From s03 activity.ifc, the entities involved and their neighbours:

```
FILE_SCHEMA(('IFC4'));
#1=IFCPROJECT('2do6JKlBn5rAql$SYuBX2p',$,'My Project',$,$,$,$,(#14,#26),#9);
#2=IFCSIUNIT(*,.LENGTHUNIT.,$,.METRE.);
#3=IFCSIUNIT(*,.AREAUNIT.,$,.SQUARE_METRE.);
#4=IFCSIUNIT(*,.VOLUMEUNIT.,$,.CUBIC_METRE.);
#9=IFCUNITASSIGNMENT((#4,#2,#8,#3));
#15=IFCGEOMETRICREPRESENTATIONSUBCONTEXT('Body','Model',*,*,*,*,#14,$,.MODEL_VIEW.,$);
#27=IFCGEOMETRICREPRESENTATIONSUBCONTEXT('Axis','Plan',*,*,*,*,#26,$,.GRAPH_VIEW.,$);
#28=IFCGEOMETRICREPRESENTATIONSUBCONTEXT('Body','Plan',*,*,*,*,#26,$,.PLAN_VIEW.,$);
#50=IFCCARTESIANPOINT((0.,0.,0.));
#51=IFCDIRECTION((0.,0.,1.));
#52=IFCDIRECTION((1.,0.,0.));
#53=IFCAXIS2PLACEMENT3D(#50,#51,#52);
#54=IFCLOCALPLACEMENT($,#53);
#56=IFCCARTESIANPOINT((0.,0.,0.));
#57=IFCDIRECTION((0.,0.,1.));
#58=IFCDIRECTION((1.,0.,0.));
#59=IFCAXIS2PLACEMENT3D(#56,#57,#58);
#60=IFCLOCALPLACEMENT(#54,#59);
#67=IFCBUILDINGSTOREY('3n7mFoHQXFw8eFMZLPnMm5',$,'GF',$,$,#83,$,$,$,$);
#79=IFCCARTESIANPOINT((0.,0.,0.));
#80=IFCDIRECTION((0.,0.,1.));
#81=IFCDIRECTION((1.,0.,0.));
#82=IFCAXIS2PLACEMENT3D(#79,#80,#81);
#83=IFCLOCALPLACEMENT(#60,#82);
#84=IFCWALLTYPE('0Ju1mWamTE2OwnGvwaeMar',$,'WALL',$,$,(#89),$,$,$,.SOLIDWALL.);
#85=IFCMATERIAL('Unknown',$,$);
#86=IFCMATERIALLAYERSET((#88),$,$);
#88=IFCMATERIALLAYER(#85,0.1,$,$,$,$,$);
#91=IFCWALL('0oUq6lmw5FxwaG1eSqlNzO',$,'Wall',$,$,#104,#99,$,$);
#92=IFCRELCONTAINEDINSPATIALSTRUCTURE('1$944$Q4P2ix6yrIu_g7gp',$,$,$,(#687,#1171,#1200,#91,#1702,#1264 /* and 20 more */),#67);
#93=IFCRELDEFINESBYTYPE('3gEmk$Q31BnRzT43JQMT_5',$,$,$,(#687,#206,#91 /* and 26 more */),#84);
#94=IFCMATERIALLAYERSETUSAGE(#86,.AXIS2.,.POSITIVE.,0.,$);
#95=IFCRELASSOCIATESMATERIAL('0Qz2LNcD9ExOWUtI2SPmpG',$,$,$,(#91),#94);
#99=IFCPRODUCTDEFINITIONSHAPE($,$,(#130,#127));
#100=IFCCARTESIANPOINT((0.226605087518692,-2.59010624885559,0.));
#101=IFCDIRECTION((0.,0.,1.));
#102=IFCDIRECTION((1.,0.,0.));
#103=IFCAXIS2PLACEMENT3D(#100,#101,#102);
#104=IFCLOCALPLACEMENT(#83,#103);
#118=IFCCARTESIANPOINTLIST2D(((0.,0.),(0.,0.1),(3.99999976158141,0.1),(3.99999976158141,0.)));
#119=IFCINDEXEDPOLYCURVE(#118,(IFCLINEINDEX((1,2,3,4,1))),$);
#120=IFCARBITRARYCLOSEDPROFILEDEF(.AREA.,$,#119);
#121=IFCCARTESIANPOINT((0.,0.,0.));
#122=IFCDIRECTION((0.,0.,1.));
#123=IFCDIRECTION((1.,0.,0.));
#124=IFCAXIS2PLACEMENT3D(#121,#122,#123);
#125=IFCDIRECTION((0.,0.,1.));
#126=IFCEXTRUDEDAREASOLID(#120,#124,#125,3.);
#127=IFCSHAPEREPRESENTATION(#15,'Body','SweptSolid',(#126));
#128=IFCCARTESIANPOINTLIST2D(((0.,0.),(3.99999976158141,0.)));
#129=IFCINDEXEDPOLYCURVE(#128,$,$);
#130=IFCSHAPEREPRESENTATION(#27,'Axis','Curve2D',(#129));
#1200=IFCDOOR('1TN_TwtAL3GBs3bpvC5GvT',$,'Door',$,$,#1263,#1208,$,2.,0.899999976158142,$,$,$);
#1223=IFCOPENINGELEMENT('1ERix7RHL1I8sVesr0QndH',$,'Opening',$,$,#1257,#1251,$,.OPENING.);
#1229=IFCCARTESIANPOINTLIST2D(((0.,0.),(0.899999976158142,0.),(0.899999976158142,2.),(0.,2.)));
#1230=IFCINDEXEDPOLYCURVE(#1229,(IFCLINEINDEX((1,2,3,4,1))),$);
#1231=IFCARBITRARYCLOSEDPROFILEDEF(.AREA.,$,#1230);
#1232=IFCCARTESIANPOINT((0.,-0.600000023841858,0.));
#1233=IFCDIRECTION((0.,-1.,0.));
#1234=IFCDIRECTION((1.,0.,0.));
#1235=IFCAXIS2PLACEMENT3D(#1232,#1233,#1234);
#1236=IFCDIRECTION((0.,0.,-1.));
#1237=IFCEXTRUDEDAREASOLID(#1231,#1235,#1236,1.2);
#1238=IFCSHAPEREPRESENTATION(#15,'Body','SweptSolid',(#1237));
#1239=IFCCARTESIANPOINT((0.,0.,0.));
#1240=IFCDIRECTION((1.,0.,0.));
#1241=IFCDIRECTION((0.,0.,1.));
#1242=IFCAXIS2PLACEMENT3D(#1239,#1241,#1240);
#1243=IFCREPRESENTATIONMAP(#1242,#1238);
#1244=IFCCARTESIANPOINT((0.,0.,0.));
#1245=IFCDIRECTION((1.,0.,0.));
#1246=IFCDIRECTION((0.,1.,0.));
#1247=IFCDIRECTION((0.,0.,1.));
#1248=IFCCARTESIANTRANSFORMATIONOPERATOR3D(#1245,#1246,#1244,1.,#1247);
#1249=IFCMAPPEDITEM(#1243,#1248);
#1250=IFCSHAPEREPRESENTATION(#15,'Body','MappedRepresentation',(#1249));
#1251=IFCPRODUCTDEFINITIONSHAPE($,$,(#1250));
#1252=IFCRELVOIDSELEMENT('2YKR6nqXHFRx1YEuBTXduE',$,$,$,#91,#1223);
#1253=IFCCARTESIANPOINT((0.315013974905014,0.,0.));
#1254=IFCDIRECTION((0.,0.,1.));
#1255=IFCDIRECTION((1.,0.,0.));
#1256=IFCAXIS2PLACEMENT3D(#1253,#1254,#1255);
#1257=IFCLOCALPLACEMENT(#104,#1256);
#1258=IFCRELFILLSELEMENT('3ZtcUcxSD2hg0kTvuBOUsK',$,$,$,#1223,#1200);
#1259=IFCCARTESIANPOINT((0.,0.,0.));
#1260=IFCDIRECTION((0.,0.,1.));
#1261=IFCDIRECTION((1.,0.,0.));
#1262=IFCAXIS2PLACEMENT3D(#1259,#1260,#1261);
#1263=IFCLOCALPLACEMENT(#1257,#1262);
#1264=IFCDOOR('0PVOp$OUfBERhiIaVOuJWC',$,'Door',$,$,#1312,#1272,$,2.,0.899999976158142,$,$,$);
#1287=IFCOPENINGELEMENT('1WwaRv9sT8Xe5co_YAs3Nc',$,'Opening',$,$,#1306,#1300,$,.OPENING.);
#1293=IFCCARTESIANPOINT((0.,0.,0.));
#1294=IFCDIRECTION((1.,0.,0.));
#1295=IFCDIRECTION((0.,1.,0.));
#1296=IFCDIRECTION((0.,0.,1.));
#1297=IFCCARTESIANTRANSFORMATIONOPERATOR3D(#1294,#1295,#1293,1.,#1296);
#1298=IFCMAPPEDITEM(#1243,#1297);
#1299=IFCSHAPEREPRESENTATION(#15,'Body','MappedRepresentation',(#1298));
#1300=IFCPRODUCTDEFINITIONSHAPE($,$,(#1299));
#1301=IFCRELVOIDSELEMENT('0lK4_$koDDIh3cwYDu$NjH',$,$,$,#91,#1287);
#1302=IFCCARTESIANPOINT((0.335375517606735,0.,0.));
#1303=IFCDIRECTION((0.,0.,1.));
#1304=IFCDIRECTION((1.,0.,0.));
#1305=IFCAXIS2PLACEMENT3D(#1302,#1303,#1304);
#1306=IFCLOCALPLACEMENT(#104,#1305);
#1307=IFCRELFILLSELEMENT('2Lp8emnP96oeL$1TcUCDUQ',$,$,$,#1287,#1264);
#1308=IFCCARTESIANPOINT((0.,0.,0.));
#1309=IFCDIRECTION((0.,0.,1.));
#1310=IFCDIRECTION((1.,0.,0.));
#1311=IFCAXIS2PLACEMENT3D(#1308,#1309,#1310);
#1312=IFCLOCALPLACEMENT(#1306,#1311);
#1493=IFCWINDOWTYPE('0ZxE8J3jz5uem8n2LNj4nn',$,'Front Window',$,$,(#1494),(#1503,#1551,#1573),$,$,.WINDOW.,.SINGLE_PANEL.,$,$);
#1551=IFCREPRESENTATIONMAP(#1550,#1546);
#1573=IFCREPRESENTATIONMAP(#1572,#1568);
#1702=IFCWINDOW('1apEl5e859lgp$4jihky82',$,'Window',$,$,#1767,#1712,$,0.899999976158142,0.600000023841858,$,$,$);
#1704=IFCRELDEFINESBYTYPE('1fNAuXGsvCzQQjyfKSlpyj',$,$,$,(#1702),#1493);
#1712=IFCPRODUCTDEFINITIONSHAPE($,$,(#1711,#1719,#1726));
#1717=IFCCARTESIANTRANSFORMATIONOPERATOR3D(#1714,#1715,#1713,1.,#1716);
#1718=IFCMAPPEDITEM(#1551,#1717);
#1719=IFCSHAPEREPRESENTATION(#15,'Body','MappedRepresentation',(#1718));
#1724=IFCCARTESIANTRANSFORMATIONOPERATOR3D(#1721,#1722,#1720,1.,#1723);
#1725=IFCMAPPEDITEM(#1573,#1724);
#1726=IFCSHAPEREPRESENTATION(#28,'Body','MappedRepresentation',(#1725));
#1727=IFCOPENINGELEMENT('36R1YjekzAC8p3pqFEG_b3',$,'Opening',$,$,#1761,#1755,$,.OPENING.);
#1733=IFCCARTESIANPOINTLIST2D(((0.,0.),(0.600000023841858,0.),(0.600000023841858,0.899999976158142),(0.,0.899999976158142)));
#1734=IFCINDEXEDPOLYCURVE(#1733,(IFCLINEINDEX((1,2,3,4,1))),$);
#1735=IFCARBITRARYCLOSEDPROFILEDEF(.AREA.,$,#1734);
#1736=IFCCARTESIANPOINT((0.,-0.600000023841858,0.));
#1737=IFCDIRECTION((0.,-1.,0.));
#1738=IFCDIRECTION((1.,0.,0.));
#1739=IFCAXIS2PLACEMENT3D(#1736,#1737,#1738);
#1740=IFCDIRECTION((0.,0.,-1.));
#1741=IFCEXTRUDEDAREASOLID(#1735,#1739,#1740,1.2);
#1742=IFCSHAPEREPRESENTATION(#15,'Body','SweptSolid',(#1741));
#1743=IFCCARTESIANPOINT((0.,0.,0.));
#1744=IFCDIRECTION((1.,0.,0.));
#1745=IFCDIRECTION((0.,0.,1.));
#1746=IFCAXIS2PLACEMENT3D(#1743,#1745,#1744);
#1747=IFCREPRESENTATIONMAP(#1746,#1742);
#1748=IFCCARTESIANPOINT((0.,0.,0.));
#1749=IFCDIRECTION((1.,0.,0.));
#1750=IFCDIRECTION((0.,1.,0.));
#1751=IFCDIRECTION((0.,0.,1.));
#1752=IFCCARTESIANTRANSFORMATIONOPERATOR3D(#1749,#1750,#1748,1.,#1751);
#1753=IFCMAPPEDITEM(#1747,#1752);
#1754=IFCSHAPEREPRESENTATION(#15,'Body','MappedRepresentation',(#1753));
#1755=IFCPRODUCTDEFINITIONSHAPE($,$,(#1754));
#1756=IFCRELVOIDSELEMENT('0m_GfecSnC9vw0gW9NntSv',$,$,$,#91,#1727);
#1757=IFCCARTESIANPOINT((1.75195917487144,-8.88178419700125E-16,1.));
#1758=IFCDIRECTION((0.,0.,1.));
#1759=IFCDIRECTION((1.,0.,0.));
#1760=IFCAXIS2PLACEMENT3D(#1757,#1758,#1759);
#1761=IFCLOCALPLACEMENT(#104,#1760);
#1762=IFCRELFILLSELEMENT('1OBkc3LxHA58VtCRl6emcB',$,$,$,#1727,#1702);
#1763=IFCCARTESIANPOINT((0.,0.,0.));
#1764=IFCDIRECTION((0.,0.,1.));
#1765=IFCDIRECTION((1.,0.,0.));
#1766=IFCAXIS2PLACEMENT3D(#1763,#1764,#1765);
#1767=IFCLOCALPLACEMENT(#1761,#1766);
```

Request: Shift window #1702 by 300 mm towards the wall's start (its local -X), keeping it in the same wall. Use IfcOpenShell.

```python
import ifcopenshell
import ifcopenshell.api.geometry
import ifcopenshell.util.placement
import ifcopenshell.util.unit

model = ifcopenshell.open("s03 activity.ifc")
unit_scale = ifcopenshell.util.unit.calculate_unit_scale(model)

window = model.by_id(1702)
opening = window.FillsVoids[0].RelatingOpeningElement
wall = opening.VoidsElements[0].RelatingBuildingElement

wall_matrix = ifcopenshell.util.placement.get_local_placement(wall.ObjectPlacement)
shift = wall_matrix[:3, 0] * -0.3 / unit_scale
before = ifcopenshell.util.placement.get_local_placement(window.ObjectPlacement)[:3, 3].copy()

# The window is placed relative to its opening, so it follows when the opening moves.
matrix = ifcopenshell.util.placement.get_local_placement(opening.ObjectPlacement)
matrix[:3, 3] += shift
ifcopenshell.api.geometry.edit_object_placement(
    model, product=opening, matrix=matrix, is_si=False, should_transform_children=True
)

after = ifcopenshell.util.placement.get_local_placement(window.ObjectPlacement)[:3, 3]
print("window moved by", (after - before).round(3) + 0.0)

model.write("s03 activity_edited.ifc")
```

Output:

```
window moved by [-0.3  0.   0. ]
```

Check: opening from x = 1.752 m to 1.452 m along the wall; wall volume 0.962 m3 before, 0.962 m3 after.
